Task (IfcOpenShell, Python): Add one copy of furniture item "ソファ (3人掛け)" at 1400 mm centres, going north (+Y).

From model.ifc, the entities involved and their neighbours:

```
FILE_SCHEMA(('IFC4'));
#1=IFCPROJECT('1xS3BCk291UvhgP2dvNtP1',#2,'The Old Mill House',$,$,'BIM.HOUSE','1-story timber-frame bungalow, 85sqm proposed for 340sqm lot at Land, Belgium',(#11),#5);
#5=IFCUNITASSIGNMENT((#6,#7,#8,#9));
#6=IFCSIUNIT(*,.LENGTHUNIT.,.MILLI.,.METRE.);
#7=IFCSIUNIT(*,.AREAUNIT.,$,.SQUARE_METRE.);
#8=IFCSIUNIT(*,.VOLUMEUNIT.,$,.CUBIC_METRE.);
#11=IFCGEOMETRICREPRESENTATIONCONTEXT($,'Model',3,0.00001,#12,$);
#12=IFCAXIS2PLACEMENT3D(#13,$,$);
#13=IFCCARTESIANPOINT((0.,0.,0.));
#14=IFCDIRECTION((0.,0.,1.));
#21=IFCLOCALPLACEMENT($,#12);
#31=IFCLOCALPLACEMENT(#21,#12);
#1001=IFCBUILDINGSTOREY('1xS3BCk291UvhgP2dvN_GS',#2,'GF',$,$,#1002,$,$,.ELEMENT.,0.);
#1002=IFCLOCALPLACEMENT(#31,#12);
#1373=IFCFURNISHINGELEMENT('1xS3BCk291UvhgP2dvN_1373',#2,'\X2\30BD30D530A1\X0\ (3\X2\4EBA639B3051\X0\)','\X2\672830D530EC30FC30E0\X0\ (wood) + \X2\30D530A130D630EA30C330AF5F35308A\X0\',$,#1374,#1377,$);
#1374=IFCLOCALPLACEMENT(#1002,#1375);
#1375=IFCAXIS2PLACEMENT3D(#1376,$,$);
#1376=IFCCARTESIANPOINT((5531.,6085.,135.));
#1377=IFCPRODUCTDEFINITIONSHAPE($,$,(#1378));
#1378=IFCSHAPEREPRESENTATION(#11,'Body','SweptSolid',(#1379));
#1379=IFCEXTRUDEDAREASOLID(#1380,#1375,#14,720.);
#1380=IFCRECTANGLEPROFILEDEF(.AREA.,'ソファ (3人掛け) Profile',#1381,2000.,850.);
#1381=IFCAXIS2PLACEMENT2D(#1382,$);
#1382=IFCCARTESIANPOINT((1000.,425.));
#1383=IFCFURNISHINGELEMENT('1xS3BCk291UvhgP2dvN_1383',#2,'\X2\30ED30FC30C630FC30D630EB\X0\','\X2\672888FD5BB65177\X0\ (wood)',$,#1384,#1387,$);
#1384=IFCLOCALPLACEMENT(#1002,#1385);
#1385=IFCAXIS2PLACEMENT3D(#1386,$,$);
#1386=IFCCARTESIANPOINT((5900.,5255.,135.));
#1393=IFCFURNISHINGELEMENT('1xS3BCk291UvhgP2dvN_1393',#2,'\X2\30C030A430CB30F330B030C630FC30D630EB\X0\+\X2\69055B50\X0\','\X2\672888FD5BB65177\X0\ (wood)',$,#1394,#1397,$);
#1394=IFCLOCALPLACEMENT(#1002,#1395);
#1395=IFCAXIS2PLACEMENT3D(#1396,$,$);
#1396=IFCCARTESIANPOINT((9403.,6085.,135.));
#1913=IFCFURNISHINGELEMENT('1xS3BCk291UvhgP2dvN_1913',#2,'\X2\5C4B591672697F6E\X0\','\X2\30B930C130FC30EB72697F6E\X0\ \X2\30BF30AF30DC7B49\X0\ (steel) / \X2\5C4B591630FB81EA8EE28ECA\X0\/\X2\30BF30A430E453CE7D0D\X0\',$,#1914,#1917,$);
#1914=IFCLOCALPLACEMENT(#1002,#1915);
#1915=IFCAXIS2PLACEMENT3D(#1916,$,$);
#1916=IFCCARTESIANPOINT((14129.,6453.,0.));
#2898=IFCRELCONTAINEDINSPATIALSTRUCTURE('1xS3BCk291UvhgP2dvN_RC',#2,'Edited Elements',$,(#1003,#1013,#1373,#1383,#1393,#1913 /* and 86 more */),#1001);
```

```python
import numpy as np
import ifcopenshell
import ifcopenshell.api.geometry
import ifcopenshell.api.root
import ifcopenshell.util.element
import ifcopenshell.util.placement
import ifcopenshell.util.unit

model = ifcopenshell.open("model.ifc")
unit_scale = ifcopenshell.util.unit.calculate_unit_scale(model)


def reuse_history(source, copy):
    """copy_class also copies each property set's owner history, people and application; keep the originals."""
    for rel in copy.IsDefinedBy:
        if rel.is_a("IfcRelDefinesByProperties") and (history := rel.RelatingPropertyDefinition.OwnerHistory):
            rel.RelatingPropertyDefinition.OwnerHistory = source.OwnerHistory
            ifcopenshell.util.element.remove_deep2(model, history)


source = model.by_id(1373)
base = ifcopenshell.util.placement.get_local_placement(source.ObjectPlacement)
step = np.array([0.0, 1.0, 0.0]) * 1.4 / unit_scale

for i in range(1, 2):
    copy = ifcopenshell.api.root.copy_class(model, product=source)
    copy.Representation = ifcopenshell.util.element.copy_deep(
        model, source.Representation, exclude=["IfcGeometricRepresentationContext", "IfcRepresentationMap"]
    )
    reuse_history(source, copy)
    matrix = base.copy()
    matrix[:3, 3] += i * step
    print("added at", matrix[:3, 3].round(3) + 0.0)
    ifcopenshell.api.geometry.edit_object_placement(model, product=copy, matrix=matrix, is_si=False)

model.write("model_edited.ifc")
```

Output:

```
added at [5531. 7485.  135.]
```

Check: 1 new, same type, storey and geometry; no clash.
